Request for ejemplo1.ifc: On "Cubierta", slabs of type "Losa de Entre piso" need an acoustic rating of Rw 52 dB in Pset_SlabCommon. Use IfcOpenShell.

First a look at what the model holds.

```python
import ifcopenshell
import ifcopenshell.util.element

model = ifcopenshell.open("ejemplo1.ifc")
print(model.schema)
storey = next(s for s in model.by_type("IfcBuildingStorey") if s.Name == "Cubierta")
slabs = [e for e in ifcopenshell.util.element.get_decomposition(storey) if e.is_a("IfcSlab")]
seen = {}
for e in slabs:
    element_type = ifcopenshell.util.element.get_type(e)
    key = (element_type.Name if element_type != e and element_type else None, ifcopenshell.util.element.get_pset(e, "Pset_SlabCommon", "AcousticRating"))
    seen[key] = seen.get(key, 0) + 1
for (name, value), count in sorted(seen.items(), key=str):
    print(count, "x", name, "|", value)
```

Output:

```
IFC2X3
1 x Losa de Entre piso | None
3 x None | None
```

```python
import ifcopenshell
import ifcopenshell.api.pset
import ifcopenshell.util.element

model = ifcopenshell.open("ejemplo1.ifc")

storey = next(s for s in model.by_type("IfcBuildingStorey") if s.Name == "Cubierta")
slabs = [e for e in ifcopenshell.util.element.get_decomposition(storey) if e.is_a("IfcSlab")]

count = 0
for e in slabs:
    element_type = ifcopenshell.util.element.get_type(e)
    if element_type in (None, e) or element_type.Name != "Losa de Entre piso":
        continue
    # add_pset returns the element's existing set when there is one.
    pset = ifcopenshell.api.pset.add_pset(model, product=e, name="Pset_SlabCommon")
    ifcopenshell.api.pset.edit_pset(model, pset=pset, properties={"AcousticRating": "Rw 52 dB"})
    count += 1

print(count, "slabs updated")

model.write("ejemplo1_rev.ifc")
```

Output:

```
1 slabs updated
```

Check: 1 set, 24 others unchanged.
